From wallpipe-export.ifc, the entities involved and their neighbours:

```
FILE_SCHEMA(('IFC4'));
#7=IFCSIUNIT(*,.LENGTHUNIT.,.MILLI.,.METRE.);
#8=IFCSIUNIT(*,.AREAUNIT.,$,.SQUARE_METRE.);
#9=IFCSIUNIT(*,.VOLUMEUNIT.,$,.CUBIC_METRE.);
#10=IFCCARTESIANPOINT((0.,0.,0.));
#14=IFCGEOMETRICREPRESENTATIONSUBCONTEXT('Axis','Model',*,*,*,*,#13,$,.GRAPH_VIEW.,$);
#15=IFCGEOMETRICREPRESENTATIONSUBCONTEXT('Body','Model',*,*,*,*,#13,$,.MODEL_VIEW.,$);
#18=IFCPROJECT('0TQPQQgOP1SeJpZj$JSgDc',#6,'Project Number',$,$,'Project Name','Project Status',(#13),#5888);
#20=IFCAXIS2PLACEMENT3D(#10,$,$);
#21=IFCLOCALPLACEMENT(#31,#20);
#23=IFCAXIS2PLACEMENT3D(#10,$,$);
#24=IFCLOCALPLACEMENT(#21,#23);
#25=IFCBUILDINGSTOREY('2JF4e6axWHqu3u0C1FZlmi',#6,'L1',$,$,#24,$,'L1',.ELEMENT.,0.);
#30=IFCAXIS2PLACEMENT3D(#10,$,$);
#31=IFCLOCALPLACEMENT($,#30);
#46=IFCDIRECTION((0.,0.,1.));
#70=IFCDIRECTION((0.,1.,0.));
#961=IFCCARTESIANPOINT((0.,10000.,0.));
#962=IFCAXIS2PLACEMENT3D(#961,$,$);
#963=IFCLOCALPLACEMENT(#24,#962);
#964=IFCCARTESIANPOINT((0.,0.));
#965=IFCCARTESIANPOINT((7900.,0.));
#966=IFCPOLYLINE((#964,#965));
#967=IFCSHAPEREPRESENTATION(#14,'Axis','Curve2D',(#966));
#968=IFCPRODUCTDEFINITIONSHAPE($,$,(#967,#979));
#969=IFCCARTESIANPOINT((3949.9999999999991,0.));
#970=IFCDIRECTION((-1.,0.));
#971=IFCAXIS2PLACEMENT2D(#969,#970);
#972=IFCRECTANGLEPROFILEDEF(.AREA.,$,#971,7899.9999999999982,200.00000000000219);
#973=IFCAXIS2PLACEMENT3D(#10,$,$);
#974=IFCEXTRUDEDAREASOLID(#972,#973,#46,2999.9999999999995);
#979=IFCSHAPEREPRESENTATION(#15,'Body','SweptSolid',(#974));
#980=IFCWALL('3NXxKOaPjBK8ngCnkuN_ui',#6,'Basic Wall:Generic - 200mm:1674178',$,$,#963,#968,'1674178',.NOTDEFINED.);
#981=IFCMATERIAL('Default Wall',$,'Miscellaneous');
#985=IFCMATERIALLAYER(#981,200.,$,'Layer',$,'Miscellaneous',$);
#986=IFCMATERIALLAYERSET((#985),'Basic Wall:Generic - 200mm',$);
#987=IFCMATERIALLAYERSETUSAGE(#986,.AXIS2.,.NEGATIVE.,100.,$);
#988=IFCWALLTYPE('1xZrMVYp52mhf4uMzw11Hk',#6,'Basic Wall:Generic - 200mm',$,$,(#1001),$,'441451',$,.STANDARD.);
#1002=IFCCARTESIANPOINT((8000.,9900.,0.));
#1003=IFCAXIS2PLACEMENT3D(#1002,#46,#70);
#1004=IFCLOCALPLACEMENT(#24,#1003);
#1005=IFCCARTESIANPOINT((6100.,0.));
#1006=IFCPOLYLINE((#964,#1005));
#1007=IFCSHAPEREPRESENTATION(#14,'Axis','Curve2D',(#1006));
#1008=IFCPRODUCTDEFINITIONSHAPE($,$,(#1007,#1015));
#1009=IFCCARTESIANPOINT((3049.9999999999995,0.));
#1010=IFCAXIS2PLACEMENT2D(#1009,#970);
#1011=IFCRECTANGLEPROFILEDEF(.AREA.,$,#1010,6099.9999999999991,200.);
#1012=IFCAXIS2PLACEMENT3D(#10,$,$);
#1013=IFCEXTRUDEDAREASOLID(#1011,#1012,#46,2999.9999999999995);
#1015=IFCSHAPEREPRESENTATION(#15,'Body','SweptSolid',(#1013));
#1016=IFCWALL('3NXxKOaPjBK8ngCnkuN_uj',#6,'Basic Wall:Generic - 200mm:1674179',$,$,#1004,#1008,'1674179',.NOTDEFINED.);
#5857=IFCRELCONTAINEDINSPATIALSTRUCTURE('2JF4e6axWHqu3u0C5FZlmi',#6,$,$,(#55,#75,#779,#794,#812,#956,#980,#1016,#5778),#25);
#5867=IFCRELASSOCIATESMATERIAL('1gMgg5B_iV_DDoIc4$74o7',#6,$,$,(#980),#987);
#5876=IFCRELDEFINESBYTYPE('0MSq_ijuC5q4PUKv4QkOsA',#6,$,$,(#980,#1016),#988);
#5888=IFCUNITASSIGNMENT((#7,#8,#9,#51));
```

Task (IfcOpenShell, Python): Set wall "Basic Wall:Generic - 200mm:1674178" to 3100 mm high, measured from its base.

```python
import ifcopenshell
import ifcopenshell.geom
import ifcopenshell.util.representation
import ifcopenshell.util.shape
import ifcopenshell.util.unit

model = ifcopenshell.open("wallpipe-export.ifc")
unit_scale = ifcopenshell.util.unit.calculate_unit_scale(model)
settings = ifcopenshell.geom.settings()


def volume(element):
    """Net volume in cubic metres, openings subtracted."""
    shape = ifcopenshell.geom.create_shape(settings, element)
    return ifcopenshell.util.shape.get_volume(shape.geometry)


wall = model.by_guid("3NXxKOaPjBK8ngCnkuN_ui")
before = volume(wall)

body = ifcopenshell.util.representation.get_representation(wall, "Model", "Body")
solid = body.Items[0]
old_height = solid.Depth
solid.Depth = 3.1 / unit_scale
after = volume(wall)

print(f"height {old_height:g} -> {solid.Depth:g}, volume {before:.3f} -> {after:.3f} m3")

model.write("wallpipe-export_v2.ifc")
```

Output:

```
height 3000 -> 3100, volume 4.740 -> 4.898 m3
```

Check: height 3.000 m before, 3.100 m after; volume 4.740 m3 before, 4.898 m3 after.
